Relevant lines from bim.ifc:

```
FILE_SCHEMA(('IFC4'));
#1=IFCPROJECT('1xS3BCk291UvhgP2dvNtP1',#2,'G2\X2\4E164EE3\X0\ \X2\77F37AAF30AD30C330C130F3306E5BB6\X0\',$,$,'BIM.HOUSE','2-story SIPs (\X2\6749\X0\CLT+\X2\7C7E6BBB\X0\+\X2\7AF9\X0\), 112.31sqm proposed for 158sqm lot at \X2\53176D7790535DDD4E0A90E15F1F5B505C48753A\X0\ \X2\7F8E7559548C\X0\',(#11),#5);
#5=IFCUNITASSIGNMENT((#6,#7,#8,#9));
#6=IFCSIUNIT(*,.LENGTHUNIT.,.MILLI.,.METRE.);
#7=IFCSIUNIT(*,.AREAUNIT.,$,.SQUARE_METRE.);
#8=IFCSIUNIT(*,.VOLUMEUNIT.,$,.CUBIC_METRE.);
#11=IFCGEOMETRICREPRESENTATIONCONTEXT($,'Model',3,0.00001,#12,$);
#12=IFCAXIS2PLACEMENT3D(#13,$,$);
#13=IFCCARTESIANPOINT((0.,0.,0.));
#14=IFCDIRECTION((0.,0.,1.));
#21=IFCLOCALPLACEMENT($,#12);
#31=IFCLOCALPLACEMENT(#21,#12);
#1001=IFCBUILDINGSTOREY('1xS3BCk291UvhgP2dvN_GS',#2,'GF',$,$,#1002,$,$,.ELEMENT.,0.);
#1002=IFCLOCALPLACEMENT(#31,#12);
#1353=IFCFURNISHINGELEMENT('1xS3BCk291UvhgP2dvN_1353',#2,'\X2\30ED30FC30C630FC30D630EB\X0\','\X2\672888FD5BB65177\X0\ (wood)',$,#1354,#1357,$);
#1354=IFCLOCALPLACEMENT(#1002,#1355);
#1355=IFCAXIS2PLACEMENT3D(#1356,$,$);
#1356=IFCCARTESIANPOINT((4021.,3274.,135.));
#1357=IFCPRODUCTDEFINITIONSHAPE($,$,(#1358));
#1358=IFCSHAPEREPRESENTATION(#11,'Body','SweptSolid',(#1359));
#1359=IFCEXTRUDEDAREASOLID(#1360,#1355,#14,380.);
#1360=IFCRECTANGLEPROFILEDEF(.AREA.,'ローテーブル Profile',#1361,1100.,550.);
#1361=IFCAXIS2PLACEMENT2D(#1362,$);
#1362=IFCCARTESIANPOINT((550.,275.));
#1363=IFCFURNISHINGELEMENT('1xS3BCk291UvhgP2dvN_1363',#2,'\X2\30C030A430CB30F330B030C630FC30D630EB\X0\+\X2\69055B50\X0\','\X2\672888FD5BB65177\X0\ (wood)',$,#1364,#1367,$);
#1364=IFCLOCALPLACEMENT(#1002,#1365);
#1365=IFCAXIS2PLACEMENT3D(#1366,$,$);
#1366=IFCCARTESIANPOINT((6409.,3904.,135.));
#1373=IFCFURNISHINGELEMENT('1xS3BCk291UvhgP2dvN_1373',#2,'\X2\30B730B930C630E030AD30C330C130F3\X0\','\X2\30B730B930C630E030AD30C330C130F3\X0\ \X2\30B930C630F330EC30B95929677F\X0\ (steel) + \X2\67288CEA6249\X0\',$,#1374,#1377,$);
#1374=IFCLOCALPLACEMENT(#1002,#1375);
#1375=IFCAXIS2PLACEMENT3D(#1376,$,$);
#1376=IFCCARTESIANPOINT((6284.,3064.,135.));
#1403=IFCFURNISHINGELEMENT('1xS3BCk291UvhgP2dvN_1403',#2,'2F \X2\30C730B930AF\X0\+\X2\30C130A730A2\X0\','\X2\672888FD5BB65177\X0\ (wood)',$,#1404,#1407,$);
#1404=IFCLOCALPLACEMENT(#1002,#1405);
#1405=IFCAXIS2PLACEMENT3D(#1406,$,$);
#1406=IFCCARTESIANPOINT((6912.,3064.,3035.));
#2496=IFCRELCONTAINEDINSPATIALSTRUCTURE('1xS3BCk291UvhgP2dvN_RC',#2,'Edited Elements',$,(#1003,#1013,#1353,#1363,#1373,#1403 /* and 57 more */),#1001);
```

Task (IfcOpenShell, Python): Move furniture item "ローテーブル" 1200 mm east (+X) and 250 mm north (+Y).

```python
import ifcopenshell
import ifcopenshell.api.geometry
import ifcopenshell.util.placement

model = ifcopenshell.open("bim.ifc")

item = model.by_guid("1xS3BCk291UvhgP2dvN_1353")
matrix = ifcopenshell.util.placement.get_local_placement(item.ObjectPlacement)
matrix[0, 3] += 1200.0
matrix[1, 3] += 250.0
ifcopenshell.api.geometry.edit_object_placement(model, product=item, matrix=matrix, is_si=False)

print(ifcopenshell.util.placement.get_local_placement(item.ObjectPlacement).round(3) + 0.0)

model.write("bim_edited.ifc")
```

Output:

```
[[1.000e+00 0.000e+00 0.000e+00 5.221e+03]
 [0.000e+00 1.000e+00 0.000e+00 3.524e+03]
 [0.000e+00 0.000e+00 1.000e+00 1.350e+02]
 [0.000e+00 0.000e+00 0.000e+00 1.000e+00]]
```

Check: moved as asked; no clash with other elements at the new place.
